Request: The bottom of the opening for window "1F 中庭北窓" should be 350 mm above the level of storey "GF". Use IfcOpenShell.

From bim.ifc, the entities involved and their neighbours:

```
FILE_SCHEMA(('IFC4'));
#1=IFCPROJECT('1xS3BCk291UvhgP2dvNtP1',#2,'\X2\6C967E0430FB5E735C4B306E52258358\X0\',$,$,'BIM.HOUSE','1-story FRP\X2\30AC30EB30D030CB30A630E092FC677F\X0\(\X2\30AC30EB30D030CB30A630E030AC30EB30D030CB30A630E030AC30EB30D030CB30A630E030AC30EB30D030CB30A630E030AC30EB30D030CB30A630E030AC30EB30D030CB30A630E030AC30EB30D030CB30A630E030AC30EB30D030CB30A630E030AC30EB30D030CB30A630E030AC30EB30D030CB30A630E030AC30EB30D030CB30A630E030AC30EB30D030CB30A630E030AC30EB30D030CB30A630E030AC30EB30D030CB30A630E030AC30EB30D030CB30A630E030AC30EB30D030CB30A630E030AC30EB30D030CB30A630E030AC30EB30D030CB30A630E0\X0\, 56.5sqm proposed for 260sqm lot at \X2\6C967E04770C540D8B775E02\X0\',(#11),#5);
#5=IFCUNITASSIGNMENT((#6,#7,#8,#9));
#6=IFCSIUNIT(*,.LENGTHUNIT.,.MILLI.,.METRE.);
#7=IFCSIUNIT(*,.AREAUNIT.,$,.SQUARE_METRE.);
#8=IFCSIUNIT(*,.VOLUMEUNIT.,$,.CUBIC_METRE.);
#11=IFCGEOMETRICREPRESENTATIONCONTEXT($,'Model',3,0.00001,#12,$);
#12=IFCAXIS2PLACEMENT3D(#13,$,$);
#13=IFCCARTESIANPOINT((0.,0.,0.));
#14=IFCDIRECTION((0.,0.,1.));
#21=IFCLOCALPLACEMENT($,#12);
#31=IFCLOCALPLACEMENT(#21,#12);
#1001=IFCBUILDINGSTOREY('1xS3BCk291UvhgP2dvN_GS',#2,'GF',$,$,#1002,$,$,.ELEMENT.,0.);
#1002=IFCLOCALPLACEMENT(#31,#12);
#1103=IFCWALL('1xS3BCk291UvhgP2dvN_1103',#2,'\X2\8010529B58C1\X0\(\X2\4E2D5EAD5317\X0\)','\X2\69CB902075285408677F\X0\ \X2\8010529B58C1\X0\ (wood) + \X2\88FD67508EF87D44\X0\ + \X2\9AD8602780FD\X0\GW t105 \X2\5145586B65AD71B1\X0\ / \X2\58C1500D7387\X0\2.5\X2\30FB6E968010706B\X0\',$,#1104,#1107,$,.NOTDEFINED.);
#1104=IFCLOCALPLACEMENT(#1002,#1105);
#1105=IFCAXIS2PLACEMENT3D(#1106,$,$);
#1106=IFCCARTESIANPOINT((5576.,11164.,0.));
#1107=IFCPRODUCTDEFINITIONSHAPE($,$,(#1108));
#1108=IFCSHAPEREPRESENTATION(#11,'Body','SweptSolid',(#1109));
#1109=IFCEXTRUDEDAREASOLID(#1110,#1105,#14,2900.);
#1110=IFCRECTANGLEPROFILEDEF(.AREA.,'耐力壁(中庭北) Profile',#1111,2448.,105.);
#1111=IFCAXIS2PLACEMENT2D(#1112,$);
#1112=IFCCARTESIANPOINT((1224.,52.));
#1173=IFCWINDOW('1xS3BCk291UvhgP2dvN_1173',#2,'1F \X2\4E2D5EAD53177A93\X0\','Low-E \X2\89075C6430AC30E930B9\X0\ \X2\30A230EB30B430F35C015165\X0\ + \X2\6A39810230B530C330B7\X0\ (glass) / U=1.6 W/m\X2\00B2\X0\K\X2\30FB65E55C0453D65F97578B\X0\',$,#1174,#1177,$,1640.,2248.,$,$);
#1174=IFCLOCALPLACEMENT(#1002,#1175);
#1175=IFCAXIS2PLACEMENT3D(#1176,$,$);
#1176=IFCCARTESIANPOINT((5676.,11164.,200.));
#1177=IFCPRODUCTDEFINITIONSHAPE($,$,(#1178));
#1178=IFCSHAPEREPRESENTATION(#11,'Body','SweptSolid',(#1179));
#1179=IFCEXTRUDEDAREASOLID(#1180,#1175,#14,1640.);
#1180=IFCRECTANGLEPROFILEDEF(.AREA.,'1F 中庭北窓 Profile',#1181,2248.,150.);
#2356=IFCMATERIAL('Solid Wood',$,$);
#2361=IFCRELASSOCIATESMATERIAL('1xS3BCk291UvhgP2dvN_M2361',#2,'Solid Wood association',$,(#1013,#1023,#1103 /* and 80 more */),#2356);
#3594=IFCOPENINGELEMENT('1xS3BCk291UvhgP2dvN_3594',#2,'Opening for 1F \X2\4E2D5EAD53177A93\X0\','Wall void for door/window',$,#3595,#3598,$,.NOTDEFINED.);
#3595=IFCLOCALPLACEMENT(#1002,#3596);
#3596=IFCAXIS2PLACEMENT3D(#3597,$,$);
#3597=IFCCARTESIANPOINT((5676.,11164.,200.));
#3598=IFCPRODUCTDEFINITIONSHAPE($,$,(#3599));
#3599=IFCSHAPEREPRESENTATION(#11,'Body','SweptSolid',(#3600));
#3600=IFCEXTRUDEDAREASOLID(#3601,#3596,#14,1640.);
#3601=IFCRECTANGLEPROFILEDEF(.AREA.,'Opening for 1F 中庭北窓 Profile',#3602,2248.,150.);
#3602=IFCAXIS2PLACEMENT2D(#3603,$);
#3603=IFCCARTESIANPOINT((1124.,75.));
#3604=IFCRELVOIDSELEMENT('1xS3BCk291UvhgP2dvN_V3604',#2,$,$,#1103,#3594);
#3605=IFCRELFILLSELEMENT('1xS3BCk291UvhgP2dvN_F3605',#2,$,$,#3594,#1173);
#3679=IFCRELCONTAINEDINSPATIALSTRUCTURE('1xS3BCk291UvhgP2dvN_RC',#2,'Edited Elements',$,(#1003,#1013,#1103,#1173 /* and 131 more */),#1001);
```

```python
import numpy as np
import ifcopenshell
import ifcopenshell.api.geometry
import ifcopenshell.geom
import ifcopenshell.util.element
import ifcopenshell.util.placement
import ifcopenshell.util.shape
import ifcopenshell.util.unit

model = ifcopenshell.open("bim.ifc")
unit_scale = ifcopenshell.util.unit.calculate_unit_scale(model)

window = model.by_guid("1xS3BCk291UvhgP2dvN_1173")
opening = window.FillsVoids[0].RelatingOpeningElement
storey = ifcopenshell.util.element.get_container(window, ifc_class="IfcBuildingStorey")
level = ifcopenshell.util.placement.get_local_placement(storey.ObjectPlacement)[2, 3]

# The opening's origin need not be at the sill, so measure its lowest point.
shape = ifcopenshell.geom.create_shape(ifcopenshell.geom.settings(), opening)
bottom = ifcopenshell.util.shape.get_shape_bottom_elevation(shape, shape.geometry) / unit_scale
dz = level + 0.35 / unit_scale - bottom

shift = np.array([0.0, 0.0, dz])
# The window is not placed relative to its opening, so move both.
for product in (opening, window):
    matrix = ifcopenshell.util.placement.get_local_placement(product.ObjectPlacement)
    matrix[:3, 3] += shift
    ifcopenshell.api.geometry.edit_object_placement(model, product=product, matrix=matrix, is_si=False)

print(f"moved by {dz * unit_scale:+.3f} m")

model.write("bim_updated.ifc")
```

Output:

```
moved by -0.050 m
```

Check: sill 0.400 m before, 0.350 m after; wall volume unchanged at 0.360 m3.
